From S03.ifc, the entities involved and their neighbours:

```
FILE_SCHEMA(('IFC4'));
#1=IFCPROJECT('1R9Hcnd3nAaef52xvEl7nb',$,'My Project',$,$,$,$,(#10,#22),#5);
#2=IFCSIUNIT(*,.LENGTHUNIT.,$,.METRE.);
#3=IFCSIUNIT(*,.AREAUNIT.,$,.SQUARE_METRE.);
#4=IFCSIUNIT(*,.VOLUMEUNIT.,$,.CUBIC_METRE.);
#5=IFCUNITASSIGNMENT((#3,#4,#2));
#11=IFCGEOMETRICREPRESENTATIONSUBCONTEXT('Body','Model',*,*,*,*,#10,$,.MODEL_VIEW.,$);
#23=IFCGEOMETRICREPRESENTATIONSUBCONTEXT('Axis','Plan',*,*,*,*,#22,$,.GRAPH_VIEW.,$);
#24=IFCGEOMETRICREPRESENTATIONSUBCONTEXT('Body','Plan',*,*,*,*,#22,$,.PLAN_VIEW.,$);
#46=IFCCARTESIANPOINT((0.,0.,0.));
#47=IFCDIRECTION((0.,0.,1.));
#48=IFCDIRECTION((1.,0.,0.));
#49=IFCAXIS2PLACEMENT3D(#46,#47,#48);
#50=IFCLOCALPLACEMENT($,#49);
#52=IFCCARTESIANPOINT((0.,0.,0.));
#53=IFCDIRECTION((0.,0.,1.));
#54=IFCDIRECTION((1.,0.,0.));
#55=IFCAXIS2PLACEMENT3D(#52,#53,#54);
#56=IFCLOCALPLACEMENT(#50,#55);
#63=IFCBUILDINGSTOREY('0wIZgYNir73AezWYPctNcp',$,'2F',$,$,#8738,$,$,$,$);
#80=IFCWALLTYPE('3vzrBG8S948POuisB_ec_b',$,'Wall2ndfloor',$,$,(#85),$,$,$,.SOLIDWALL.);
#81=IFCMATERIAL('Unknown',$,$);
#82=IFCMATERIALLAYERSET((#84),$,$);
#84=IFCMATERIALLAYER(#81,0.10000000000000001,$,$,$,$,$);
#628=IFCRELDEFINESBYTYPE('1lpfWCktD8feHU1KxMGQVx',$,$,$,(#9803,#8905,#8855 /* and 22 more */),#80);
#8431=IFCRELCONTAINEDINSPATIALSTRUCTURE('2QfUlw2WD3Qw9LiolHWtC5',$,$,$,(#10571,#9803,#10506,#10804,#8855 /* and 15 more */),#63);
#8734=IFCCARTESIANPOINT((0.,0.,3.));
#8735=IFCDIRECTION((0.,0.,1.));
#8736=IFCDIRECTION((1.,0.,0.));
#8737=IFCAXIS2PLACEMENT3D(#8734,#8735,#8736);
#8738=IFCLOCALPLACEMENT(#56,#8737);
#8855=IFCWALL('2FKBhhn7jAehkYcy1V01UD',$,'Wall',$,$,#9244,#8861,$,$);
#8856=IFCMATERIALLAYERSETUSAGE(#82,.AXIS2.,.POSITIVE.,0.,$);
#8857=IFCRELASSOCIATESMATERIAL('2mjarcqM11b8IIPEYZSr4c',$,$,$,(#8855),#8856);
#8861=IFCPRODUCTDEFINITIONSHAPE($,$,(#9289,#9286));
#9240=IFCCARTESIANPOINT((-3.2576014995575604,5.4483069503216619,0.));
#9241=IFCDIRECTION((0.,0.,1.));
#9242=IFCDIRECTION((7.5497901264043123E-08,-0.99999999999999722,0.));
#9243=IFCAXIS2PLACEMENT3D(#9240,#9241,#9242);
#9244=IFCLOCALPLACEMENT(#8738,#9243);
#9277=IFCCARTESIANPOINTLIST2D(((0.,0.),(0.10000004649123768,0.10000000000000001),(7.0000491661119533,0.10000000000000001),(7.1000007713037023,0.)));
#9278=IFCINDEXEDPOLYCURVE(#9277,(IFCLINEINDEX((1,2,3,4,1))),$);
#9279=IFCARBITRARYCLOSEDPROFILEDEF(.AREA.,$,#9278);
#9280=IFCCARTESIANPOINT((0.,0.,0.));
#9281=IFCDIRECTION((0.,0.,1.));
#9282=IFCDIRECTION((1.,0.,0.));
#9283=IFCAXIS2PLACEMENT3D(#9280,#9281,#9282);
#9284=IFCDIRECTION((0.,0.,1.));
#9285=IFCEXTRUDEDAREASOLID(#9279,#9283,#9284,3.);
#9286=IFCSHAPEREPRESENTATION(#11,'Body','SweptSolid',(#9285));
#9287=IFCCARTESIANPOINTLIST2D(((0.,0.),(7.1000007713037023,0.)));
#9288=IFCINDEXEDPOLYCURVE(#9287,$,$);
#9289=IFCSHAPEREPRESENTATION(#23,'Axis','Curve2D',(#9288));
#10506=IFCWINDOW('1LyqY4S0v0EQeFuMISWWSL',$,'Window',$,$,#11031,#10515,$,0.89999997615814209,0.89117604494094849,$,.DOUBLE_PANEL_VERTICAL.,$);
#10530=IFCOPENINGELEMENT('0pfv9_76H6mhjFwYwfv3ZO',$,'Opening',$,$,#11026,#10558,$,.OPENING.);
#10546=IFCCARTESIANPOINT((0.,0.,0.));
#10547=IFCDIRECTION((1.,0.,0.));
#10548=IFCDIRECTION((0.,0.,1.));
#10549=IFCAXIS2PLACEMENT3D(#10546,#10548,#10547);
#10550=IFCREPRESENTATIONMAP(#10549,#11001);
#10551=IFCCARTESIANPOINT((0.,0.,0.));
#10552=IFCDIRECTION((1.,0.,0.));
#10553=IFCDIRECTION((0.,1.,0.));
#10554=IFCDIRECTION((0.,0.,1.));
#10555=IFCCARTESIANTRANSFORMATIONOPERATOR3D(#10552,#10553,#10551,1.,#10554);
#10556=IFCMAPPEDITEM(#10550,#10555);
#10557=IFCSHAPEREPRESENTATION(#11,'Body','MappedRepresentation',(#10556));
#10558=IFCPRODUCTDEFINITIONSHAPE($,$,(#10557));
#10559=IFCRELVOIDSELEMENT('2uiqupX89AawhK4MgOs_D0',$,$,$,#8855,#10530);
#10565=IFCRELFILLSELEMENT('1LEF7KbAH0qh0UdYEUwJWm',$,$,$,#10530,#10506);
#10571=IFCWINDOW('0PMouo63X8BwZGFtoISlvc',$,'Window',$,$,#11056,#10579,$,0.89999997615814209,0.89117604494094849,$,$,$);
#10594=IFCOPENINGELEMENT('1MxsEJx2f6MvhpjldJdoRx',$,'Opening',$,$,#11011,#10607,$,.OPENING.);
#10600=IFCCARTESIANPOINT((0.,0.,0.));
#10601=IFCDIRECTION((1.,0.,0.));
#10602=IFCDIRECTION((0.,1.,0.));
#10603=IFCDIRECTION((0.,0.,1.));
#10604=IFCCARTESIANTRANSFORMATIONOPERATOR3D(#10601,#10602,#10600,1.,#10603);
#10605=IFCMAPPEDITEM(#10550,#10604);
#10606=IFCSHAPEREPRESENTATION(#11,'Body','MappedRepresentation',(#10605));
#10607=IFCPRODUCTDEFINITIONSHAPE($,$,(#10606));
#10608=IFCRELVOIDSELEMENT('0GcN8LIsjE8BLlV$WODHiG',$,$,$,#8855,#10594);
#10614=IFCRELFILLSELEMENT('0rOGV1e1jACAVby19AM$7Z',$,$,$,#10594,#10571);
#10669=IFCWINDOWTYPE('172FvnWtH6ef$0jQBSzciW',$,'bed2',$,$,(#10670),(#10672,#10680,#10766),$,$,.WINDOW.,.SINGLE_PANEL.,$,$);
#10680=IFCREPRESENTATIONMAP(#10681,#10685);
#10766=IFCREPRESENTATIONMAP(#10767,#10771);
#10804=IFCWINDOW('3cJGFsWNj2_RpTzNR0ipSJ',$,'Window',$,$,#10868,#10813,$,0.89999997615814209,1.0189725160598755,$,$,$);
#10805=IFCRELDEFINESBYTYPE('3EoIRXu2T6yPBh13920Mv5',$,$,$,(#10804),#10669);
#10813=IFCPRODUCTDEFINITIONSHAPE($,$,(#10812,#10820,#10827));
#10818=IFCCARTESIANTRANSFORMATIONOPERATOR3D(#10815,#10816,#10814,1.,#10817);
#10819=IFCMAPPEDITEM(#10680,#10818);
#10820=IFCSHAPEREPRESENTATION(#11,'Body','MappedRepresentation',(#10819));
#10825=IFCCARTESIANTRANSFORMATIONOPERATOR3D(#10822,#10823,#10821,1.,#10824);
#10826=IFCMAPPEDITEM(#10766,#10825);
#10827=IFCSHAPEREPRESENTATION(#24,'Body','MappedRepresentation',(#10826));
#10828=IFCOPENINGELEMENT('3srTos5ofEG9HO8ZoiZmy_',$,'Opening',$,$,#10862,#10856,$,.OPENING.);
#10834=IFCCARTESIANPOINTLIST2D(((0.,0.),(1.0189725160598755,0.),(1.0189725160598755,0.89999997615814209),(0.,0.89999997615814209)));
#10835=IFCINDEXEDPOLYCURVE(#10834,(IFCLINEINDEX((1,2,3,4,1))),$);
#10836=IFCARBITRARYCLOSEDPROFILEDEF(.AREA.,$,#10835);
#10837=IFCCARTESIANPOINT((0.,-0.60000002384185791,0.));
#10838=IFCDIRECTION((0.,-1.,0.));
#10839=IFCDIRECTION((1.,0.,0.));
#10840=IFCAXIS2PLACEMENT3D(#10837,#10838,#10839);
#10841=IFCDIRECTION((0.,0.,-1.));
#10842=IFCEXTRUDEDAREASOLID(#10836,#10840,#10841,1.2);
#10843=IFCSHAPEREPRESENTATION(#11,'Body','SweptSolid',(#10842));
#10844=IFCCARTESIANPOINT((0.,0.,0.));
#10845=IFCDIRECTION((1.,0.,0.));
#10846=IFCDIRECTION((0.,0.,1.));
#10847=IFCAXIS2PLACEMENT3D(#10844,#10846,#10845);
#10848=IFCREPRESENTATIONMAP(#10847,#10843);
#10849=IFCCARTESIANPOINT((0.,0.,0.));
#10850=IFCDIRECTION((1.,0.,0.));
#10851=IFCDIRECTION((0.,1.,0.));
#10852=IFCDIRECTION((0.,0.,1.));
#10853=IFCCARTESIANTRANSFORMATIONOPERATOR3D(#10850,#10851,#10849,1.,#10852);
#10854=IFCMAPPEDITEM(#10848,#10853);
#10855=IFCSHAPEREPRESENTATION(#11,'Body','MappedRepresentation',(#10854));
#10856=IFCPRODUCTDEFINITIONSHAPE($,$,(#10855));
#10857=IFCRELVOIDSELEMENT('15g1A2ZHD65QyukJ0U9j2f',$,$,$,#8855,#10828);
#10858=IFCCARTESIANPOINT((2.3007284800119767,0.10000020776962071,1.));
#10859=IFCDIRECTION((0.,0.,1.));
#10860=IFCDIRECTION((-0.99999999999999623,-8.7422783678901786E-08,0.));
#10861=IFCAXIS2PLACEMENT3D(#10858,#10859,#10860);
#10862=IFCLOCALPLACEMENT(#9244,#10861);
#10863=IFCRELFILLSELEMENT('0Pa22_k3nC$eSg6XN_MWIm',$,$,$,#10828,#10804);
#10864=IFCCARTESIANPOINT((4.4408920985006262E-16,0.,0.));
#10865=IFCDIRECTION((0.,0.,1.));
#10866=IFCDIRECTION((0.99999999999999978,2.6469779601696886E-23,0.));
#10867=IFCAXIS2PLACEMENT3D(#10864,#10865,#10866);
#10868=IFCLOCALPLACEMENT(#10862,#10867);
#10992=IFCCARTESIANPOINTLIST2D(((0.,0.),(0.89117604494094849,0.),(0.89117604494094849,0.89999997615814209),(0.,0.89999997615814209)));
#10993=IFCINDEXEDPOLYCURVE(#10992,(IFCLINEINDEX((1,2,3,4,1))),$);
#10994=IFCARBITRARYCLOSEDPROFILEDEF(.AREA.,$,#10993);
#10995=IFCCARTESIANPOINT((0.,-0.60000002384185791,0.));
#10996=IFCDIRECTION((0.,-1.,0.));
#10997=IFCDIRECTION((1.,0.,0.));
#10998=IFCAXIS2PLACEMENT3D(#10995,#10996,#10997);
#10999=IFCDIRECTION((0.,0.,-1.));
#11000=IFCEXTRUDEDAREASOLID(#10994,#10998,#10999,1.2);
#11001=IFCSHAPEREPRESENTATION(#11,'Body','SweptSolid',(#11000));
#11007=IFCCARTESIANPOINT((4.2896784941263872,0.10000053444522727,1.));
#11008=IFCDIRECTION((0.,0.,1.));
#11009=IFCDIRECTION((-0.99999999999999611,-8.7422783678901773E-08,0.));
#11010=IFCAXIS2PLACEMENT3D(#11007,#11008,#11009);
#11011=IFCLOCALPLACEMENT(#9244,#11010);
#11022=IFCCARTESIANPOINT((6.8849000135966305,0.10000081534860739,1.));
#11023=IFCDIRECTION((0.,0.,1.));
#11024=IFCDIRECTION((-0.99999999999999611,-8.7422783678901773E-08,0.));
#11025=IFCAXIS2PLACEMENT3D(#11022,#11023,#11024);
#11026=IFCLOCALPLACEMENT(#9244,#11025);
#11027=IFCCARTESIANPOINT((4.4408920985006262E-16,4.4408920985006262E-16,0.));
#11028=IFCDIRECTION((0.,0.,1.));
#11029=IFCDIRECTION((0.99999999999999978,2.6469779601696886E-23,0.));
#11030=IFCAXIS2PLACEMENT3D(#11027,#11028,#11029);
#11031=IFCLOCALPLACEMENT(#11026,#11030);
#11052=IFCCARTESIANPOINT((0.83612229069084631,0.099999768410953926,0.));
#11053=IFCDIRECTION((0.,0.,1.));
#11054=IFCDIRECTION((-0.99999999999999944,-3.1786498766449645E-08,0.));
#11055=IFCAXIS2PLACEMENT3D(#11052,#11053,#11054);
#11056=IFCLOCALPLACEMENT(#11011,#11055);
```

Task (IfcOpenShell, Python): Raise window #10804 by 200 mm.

```python
import numpy as np
import ifcopenshell
import ifcopenshell.api.geometry
import ifcopenshell.util.placement
import ifcopenshell.util.unit

model = ifcopenshell.open("S03.ifc")
unit_scale = ifcopenshell.util.unit.calculate_unit_scale(model)

window = model.by_guid("3cJGFsWNj2_RpTzNR0ipSJ")
opening = window.FillsVoids[0].RelatingOpeningElement
dz = 0.2 / unit_scale

shift = np.array([0.0, 0.0, dz])
# The window is placed relative to its opening, so it follows when the opening moves.
matrix = ifcopenshell.util.placement.get_local_placement(opening.ObjectPlacement)
matrix[:3, 3] += shift
ifcopenshell.api.geometry.edit_object_placement(
    model, product=opening, matrix=matrix, is_si=False, should_transform_children=True
)

print(f"moved by {dz * unit_scale:+.3f} m")

model.write("S03-out.ifc")
```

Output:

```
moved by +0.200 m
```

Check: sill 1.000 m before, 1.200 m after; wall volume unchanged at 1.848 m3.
